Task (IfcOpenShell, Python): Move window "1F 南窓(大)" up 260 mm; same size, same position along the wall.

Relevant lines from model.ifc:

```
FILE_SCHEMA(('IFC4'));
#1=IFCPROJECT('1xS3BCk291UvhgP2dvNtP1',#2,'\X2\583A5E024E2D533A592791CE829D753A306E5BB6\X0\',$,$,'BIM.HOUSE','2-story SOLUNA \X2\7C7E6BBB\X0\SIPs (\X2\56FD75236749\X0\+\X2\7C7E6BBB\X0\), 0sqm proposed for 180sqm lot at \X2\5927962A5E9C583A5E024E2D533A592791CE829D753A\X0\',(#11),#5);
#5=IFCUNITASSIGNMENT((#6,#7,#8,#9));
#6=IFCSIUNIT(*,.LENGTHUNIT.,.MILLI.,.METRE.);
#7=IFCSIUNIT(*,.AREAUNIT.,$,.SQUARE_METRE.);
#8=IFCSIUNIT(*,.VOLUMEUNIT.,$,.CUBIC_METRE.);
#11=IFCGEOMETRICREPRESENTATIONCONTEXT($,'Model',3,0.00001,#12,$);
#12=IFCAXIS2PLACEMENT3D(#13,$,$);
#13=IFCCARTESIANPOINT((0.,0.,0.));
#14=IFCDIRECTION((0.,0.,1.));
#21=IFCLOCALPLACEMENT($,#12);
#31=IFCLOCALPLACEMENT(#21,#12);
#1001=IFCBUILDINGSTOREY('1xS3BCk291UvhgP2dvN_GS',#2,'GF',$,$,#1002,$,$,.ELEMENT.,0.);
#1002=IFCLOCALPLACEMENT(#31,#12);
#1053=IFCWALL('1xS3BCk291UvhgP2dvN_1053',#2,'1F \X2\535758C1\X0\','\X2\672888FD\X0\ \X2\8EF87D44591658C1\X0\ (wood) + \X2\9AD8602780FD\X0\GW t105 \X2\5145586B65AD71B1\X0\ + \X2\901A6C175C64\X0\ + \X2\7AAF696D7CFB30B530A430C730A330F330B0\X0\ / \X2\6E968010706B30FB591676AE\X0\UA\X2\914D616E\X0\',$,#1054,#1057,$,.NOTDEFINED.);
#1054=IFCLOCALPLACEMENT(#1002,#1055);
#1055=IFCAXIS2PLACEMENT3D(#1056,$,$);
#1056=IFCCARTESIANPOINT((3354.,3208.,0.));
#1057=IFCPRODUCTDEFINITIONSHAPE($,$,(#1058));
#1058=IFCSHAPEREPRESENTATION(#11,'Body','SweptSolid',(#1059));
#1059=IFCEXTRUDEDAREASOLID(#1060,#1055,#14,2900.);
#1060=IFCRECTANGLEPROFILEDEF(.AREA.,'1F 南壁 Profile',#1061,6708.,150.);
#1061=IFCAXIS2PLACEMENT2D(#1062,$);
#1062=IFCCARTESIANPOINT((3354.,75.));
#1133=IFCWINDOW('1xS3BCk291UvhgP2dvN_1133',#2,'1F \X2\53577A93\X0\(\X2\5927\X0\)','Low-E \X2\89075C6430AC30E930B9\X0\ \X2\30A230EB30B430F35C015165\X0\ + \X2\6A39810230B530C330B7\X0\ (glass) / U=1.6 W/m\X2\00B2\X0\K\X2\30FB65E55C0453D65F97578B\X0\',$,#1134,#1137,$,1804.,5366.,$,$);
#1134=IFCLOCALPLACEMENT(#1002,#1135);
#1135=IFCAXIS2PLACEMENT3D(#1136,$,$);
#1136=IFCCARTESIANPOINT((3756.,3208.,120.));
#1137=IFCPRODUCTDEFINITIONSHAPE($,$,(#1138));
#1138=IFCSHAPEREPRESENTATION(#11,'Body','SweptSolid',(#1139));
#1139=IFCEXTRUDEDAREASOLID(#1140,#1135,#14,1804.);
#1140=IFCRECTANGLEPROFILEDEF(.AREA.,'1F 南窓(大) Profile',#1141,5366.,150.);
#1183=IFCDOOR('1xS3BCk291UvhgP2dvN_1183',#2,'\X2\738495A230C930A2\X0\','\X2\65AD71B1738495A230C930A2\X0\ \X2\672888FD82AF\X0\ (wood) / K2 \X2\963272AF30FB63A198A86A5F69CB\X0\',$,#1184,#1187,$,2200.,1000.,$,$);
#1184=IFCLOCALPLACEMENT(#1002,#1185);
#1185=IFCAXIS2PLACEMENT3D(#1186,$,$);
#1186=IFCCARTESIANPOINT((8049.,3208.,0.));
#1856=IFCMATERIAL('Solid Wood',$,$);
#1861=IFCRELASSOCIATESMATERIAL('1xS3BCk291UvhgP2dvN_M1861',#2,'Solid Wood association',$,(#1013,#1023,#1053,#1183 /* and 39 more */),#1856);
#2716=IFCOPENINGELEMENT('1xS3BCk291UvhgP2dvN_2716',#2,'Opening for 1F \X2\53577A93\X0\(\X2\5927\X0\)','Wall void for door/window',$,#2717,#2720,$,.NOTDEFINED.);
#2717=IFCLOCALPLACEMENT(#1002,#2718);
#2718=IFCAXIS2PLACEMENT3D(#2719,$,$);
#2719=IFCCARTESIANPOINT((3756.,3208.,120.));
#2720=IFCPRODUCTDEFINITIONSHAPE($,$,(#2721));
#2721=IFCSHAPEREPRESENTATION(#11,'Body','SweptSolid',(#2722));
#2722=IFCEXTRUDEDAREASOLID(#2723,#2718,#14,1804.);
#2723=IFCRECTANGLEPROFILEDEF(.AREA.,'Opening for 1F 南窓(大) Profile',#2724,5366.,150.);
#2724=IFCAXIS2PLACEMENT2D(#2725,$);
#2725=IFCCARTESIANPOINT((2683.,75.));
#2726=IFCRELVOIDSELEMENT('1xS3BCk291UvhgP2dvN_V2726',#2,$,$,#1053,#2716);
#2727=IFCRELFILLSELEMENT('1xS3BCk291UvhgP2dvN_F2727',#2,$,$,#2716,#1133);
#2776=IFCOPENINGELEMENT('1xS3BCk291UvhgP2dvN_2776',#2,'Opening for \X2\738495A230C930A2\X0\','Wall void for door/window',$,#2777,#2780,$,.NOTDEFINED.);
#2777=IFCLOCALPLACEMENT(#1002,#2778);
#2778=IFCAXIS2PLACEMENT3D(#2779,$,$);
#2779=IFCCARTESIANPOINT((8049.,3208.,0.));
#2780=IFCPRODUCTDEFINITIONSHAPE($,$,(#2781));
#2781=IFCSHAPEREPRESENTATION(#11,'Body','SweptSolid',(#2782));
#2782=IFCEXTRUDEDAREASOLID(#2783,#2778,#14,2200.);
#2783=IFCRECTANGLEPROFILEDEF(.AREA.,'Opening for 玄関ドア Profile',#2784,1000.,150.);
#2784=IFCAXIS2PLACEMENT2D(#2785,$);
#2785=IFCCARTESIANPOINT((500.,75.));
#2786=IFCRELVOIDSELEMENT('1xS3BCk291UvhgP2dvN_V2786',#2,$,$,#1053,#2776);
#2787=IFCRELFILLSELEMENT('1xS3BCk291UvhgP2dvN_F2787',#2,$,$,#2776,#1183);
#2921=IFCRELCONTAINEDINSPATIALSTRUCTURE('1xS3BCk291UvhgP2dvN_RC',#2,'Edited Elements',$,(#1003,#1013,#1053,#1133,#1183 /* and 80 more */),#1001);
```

```python
import numpy as np
import ifcopenshell
import ifcopenshell.api.geometry
import ifcopenshell.util.placement
import ifcopenshell.util.unit

model = ifcopenshell.open("model.ifc")
unit_scale = ifcopenshell.util.unit.calculate_unit_scale(model)

window = model.by_id(1133)
opening = window.FillsVoids[0].RelatingOpeningElement
dz = 0.26 / unit_scale

shift = np.array([0.0, 0.0, dz])
# The window is not placed relative to its opening, so move both.
for product in (opening, window):
    matrix = ifcopenshell.util.placement.get_local_placement(product.ObjectPlacement)
    matrix[:3, 3] += shift
    ifcopenshell.api.geometry.edit_object_placement(model, product=product, matrix=matrix, is_si=False)

print(f"moved by {dz * unit_scale:+.3f} m")

model.write("model_edited.ifc")
```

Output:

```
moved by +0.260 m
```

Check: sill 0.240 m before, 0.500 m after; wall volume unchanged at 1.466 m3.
